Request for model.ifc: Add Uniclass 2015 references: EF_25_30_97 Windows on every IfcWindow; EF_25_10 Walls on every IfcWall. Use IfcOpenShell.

First a look at what the model holds.

```python
import ifcopenshell

model = ifcopenshell.open("model.ifc")
print(model.schema)
print("classifications:", [c.Name for c in model.by_type("IfcClassification")])
for ifc_class in ("IfcDoor", "IfcRoof", "IfcStair", "IfcWall", "IfcWindow"):
    print(ifc_class, len(model.by_type(ifc_class)))
```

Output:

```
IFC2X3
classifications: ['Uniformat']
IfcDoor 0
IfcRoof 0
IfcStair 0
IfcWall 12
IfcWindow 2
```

```python
import ifcopenshell
import ifcopenshell.api.classification

model = ifcopenshell.open("model.ifc")

# IFC2X3 requires Source and Edition and has no link from the project to the system.
system = model.create_entity("IfcClassification", Source="NBS", Edition="2015", Name="Uniclass 2015")

codes = {
    "IfcWindow": ("EF_25_30_97", "Windows"),
    "IfcWall": ("EF_25_10", "Walls"),
}
for ifc_class, (code, name) in codes.items():
    products = model.by_type(ifc_class)
    ifcopenshell.api.classification.add_reference(
        model, products=products, classification=system, identification=code, name=name
    )
    print(code, len(products))

model.write("model_v2.ifc")
```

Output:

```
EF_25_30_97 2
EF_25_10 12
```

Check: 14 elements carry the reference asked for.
